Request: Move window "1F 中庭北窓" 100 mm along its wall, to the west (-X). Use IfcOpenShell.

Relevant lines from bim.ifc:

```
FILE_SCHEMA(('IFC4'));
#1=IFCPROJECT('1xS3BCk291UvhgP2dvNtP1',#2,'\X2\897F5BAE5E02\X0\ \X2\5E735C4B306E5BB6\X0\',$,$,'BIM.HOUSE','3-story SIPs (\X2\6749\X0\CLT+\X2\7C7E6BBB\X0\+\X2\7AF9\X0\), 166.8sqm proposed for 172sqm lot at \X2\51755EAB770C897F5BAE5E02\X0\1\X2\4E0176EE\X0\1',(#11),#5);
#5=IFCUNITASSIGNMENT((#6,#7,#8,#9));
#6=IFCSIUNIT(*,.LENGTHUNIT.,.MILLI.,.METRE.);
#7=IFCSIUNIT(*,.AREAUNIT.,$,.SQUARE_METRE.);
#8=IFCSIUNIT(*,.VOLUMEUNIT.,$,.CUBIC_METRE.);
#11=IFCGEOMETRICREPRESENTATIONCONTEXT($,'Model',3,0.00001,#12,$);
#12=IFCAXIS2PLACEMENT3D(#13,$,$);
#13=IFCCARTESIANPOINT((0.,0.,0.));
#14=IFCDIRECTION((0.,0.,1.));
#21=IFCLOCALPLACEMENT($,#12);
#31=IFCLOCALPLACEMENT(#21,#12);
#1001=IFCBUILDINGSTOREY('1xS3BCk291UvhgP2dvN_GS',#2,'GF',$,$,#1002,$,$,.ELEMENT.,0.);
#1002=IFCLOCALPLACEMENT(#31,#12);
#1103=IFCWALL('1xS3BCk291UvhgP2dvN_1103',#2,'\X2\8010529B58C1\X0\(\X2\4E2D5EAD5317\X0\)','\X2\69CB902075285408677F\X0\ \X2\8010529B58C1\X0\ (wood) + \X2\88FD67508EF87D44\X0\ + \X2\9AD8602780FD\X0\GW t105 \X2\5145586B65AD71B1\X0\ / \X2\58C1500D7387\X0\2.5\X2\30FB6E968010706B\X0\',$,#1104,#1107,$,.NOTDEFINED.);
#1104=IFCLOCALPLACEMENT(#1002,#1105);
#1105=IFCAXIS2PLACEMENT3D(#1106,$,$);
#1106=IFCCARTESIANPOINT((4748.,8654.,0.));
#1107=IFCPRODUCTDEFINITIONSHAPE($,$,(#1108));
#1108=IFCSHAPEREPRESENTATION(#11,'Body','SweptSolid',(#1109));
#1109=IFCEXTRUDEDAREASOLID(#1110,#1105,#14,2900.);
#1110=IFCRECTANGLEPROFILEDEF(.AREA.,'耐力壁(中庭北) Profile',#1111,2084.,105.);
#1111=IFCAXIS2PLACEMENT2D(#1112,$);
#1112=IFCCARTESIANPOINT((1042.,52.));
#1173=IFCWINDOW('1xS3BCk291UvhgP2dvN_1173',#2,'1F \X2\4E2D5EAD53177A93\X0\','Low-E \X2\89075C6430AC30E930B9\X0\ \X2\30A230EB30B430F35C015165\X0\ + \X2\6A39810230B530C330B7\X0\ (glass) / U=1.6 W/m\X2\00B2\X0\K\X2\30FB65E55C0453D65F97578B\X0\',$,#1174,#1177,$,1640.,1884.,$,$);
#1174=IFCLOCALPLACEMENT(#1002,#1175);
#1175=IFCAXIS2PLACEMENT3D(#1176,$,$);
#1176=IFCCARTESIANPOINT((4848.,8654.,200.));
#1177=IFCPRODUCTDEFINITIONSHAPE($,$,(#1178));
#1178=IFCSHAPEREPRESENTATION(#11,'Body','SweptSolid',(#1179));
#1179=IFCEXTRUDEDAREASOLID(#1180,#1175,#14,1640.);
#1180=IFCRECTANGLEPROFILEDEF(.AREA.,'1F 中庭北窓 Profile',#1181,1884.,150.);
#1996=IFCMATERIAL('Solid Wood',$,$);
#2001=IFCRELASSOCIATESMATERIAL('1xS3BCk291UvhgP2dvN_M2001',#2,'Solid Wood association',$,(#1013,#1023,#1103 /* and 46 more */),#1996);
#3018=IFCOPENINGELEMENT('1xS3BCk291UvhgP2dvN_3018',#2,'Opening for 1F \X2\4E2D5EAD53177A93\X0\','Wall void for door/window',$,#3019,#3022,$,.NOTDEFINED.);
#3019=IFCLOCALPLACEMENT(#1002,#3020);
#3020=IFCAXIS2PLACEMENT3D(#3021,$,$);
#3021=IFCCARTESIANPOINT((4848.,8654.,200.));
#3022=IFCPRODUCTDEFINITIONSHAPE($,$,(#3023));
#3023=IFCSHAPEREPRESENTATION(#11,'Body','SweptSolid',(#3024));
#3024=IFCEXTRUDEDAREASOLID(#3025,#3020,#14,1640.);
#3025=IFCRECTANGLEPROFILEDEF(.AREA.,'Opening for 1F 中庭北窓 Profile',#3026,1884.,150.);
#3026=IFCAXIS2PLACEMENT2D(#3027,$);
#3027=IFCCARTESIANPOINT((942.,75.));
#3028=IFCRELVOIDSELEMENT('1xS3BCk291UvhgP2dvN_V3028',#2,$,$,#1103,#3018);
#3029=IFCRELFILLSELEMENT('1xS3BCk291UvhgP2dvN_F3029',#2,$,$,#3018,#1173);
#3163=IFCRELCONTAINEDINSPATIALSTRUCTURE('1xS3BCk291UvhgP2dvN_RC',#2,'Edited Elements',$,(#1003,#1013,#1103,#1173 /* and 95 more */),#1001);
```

```python
import ifcopenshell
import ifcopenshell.api.geometry
import ifcopenshell.util.placement

model = ifcopenshell.open("bim.ifc")

window = model.by_id(1173)
opening = window.FillsVoids[0].RelatingOpeningElement
wall = opening.VoidsElements[0].RelatingBuildingElement

wall_matrix = ifcopenshell.util.placement.get_local_placement(wall.ObjectPlacement)
shift = wall_matrix[:3, 0] * -100.0
before = ifcopenshell.util.placement.get_local_placement(window.ObjectPlacement)[:3, 3].copy()

# The window is not placed relative to its opening, so move both.
for product in (opening, window):
    matrix = ifcopenshell.util.placement.get_local_placement(product.ObjectPlacement)
    matrix[:3, 3] += shift
    ifcopenshell.api.geometry.edit_object_placement(model, product=product, matrix=matrix, is_si=False)

after = ifcopenshell.util.placement.get_local_placement(window.ObjectPlacement)[:3, 3]
print("window moved by", (after - before).round(3) + 0.0)

model.write("bim_updated.ifc")
```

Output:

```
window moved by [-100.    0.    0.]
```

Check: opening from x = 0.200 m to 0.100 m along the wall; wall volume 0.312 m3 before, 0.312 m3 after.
